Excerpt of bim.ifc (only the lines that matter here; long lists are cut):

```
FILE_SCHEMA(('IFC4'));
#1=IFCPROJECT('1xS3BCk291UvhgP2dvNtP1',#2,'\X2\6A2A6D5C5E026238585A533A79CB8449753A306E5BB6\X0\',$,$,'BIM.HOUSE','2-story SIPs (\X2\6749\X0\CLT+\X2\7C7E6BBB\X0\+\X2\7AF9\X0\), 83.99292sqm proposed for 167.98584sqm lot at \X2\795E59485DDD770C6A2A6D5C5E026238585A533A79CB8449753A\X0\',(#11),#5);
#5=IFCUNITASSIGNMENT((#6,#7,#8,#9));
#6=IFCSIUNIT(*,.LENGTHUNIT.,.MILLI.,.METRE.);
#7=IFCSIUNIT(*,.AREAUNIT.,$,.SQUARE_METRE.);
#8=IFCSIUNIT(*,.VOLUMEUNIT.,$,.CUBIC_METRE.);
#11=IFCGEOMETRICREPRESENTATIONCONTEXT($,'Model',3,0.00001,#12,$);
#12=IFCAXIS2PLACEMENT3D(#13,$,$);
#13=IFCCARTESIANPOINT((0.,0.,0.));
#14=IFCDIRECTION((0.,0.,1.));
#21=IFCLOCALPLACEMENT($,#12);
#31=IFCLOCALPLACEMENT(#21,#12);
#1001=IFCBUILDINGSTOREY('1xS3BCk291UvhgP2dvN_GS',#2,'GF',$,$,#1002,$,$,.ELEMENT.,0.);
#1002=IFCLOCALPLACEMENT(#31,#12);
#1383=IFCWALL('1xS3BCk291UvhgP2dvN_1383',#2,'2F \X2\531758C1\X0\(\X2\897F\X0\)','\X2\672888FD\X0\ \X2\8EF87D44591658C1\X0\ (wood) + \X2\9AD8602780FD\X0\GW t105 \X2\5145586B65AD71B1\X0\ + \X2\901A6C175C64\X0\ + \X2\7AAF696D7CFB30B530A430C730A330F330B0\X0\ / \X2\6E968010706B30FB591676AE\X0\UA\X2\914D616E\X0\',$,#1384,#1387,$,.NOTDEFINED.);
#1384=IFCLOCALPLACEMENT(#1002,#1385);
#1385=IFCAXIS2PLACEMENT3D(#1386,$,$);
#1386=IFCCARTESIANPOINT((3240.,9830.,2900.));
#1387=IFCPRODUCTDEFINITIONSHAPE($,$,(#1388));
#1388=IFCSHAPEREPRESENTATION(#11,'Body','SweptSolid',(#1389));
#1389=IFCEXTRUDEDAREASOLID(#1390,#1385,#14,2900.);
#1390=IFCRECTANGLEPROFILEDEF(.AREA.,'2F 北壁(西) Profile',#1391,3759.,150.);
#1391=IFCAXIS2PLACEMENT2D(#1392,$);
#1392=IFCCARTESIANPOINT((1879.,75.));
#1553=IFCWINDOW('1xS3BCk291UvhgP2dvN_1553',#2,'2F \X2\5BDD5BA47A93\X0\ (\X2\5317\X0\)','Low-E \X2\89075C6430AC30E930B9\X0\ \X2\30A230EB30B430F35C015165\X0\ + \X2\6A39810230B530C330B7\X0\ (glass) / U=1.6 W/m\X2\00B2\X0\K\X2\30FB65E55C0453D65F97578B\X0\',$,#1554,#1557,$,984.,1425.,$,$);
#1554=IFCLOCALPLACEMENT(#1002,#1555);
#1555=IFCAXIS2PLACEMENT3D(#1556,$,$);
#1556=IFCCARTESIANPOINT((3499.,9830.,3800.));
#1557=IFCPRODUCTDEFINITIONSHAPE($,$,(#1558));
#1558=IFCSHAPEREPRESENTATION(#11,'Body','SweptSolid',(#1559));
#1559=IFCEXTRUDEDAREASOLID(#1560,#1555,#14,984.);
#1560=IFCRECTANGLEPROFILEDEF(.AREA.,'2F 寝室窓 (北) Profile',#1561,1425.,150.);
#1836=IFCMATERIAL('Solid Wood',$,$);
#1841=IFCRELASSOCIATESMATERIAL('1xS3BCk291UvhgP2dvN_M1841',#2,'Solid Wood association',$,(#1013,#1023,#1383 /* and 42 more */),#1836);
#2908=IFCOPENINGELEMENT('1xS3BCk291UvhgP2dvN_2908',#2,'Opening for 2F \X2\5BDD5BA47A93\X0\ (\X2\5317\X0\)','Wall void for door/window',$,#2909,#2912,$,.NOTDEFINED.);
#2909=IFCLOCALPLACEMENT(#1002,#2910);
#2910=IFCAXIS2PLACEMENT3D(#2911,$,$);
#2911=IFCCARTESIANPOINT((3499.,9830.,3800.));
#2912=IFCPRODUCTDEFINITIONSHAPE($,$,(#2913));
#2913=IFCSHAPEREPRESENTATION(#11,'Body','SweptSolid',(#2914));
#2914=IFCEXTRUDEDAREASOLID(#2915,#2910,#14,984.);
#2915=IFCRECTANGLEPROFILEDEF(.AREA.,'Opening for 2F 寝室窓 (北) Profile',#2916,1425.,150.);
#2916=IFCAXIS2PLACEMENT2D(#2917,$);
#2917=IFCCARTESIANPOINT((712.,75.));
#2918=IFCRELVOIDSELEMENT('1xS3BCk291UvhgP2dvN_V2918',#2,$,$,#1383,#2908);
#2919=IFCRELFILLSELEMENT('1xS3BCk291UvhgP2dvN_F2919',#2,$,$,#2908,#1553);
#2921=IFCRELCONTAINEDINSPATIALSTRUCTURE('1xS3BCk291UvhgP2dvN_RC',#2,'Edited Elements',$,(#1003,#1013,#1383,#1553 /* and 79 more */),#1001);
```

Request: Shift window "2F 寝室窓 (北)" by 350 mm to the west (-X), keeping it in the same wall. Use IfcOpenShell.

```python
import ifcopenshell
import ifcopenshell.api.geometry
import ifcopenshell.util.placement
import ifcopenshell.util.unit

model = ifcopenshell.open("bim.ifc")
unit_scale = ifcopenshell.util.unit.calculate_unit_scale(model)

window = model.by_guid("1xS3BCk291UvhgP2dvN_1553")
opening = window.FillsVoids[0].RelatingOpeningElement
wall = opening.VoidsElements[0].RelatingBuildingElement

wall_matrix = ifcopenshell.util.placement.get_local_placement(wall.ObjectPlacement)
shift = wall_matrix[:3, 0] * -0.35 / unit_scale
before = ifcopenshell.util.placement.get_local_placement(window.ObjectPlacement)[:3, 3].copy()

# The window is not placed relative to its opening, so move both.
for product in (opening, window):
    matrix = ifcopenshell.util.placement.get_local_placement(product.ObjectPlacement)
    matrix[:3, 3] += shift
    ifcopenshell.api.geometry.edit_object_placement(model, product=product, matrix=matrix, is_si=False)

after = ifcopenshell.util.placement.get_local_placement(window.ObjectPlacement)[:3, 3]
print("window moved by", (after - before).round(3) + 0.0)

model.write("bim-out.ifc")
```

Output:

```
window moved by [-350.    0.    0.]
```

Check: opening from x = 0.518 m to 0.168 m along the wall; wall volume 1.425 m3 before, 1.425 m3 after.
